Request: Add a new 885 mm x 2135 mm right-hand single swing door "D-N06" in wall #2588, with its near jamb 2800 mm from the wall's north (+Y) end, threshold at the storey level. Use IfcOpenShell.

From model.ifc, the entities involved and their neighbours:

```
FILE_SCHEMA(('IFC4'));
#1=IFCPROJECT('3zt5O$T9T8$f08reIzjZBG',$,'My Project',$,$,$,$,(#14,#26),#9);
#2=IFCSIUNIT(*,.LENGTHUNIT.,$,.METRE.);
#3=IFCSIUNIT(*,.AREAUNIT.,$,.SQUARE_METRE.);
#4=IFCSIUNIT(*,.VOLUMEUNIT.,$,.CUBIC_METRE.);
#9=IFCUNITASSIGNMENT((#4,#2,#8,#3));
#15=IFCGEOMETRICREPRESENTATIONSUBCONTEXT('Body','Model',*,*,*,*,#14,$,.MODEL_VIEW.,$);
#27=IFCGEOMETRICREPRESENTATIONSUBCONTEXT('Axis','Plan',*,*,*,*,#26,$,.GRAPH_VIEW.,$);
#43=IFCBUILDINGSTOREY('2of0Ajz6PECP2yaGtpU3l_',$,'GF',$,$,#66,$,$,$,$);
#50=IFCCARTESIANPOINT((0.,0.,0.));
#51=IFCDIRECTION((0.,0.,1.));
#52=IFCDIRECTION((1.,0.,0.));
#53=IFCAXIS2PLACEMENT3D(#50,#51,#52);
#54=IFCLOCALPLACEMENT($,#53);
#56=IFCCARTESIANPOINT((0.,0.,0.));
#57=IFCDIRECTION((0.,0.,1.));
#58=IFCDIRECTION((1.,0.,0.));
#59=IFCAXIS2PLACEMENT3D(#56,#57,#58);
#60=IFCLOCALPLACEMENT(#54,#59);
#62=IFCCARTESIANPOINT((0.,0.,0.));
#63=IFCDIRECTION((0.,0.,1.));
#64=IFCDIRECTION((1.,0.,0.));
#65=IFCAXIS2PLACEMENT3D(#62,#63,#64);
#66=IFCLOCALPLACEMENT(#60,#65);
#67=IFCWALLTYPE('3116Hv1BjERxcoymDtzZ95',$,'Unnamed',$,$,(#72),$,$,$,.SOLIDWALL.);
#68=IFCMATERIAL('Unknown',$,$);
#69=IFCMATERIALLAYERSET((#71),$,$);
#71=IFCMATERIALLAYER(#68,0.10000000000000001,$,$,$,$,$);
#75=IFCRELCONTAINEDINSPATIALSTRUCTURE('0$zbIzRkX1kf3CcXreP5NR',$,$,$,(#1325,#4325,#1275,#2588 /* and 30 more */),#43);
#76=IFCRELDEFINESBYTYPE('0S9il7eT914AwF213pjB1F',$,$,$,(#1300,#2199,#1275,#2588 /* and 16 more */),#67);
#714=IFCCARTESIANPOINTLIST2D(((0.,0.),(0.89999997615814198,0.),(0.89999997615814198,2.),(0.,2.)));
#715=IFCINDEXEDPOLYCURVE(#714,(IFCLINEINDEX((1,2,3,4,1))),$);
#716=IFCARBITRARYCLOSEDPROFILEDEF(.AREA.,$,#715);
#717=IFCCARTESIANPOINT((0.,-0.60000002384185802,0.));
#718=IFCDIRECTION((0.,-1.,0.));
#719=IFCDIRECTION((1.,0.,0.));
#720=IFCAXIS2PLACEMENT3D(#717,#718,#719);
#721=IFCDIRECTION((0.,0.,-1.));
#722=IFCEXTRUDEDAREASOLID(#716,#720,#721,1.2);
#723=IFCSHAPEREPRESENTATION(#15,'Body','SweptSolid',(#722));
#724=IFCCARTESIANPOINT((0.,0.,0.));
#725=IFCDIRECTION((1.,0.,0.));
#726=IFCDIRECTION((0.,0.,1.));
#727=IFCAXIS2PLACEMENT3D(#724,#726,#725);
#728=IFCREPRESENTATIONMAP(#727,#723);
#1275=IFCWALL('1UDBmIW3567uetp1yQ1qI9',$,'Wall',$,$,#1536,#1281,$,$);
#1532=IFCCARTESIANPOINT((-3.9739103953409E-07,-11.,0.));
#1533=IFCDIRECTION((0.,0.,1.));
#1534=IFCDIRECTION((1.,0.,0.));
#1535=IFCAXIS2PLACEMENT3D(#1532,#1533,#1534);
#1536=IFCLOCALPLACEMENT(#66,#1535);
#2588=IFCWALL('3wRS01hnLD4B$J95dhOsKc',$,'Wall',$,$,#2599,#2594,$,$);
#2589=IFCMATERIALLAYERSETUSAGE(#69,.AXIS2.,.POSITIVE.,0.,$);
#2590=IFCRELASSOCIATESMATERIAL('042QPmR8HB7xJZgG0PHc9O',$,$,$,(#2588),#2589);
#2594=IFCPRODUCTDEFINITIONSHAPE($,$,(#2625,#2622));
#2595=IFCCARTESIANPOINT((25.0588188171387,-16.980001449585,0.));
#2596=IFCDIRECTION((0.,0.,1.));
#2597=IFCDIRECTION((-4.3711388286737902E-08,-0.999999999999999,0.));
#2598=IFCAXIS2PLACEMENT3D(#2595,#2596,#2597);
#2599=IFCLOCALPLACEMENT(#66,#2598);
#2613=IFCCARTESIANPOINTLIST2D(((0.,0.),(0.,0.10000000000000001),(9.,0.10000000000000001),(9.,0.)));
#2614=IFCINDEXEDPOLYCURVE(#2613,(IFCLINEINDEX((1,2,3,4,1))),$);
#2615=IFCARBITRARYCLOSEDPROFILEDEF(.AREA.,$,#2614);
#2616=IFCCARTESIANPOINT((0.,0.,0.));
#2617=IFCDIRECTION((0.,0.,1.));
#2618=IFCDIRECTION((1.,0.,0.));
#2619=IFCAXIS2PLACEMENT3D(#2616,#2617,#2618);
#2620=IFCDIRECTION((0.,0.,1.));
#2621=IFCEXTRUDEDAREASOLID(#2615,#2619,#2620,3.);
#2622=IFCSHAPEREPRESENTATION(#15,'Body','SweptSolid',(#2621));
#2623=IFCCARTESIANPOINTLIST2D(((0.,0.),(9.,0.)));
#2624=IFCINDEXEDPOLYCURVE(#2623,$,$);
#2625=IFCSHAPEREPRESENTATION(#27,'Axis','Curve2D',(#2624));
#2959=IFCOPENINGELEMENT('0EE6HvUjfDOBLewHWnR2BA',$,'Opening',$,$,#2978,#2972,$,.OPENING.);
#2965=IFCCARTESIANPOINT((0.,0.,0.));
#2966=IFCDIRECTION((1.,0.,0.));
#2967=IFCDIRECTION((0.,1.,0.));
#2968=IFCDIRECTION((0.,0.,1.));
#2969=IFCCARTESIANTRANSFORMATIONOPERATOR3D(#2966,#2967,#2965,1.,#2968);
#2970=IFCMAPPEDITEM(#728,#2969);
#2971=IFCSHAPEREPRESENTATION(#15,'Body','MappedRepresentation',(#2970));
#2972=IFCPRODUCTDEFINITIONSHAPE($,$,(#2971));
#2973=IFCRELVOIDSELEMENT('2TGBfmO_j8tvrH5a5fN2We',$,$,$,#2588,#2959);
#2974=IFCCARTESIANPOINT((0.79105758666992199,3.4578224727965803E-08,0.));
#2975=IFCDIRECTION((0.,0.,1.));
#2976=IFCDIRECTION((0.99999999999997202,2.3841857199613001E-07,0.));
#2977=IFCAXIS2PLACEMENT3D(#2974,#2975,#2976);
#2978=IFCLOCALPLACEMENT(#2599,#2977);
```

```python
import numpy as np
import ifcopenshell
import ifcopenshell.api.feature
import ifcopenshell.api.geometry
import ifcopenshell.api.root
import ifcopenshell.api.spatial
import ifcopenshell.geom
import ifcopenshell.util.element
import ifcopenshell.util.placement
import ifcopenshell.util.representation
import ifcopenshell.util.shape
import ifcopenshell.util.unit

model = ifcopenshell.open("model.ifc")
unit_scale = ifcopenshell.util.unit.calculate_unit_scale(model)
settings = ifcopenshell.geom.settings()


def volume(element):
    """Net volume in cubic metres, openings subtracted."""
    shape = ifcopenshell.geom.create_shape(settings, element)
    return ifcopenshell.util.shape.get_volume(shape.geometry)


wall = model.by_id(2588)
storey = ifcopenshell.util.element.get_container(wall, ifc_class="IfcBuildingStorey")
context = ifcopenshell.util.representation.get_context(model, "Model", "Body", "MODEL_VIEW")
before = volume(wall)

width, height, from_end, sill = 0.885, 2.135, 2.8, 0.0  # metres

# The wall runs along its own X axis, and the end named is its -X end.
wall_shape = ifcopenshell.geom.create_shape(settings, wall)
x, y, z = ifcopenshell.util.shape.get_vertices(wall_shape.geometry).T
start = x.min() + from_end
face, thickness = float(y.min()), float(y.max() - y.min())
wall_matrix = ifcopenshell.util.placement.get_local_placement(wall.ObjectPlacement)
level = ifcopenshell.util.placement.get_local_placement(storey.ObjectPlacement)[2, 3]


def in_wall(x, y):
    """Placement at x, y metres in the wall's axes, at sill height."""
    matrix = wall_matrix.copy()
    matrix[:, 3] = wall_matrix @ np.array([x / unit_scale, y / unit_scale, 0.0, 1.0])
    matrix[2, 3] = level + sill / unit_scale
    return matrix


# Opening: a box that overshoots both wall faces by 50 mm.
opening = ifcopenshell.api.root.create_entity(model, ifc_class="IfcOpeningElement", predefined_type="OPENING")
box = ifcopenshell.api.geometry.add_wall_representation(
    model, context=context, length=width, height=height, thickness=thickness + 0.1
)
ifcopenshell.api.geometry.assign_representation(model, product=opening, representation=box)
ifcopenshell.api.geometry.edit_object_placement(model, product=opening, matrix=in_wall(start, face - 0.05), is_si=False)
ifcopenshell.api.feature.add_feature(model, feature=opening, element=wall)

door = ifcopenshell.api.root.create_entity(model, ifc_class="IfcDoor", name="D-N06", predefined_type="DOOR")
door.OverallWidth, door.OverallHeight = width / unit_scale, height / unit_scale
door.OperationType = "SINGLE_SWING_RIGHT"
body = ifcopenshell.api.geometry.add_door_representation(
    model,
    context=context,
    overall_width=door.OverallWidth,
    overall_height=door.OverallHeight,
    operation_type="SINGLE_SWING_RIGHT",
    lining_properties={"LiningDepth": thickness / unit_scale, "ThresholdDepth": thickness / unit_scale},
)
ifcopenshell.api.geometry.assign_representation(model, product=door, representation=body)
ifcopenshell.api.spatial.assign_container(model, products=[door], relating_structure=storey)
ifcopenshell.api.feature.add_filling(model, opening=opening, element=door)

# The lining spans the wall, so the door starts at the wall face.
ifcopenshell.api.geometry.edit_object_placement(model, product=door, matrix=in_wall(start, face), is_si=False)

after = volume(wall)

print(f"wall volume {before:.3f} -> {after:.3f} m3")

model.write("model_updated.ifc")
```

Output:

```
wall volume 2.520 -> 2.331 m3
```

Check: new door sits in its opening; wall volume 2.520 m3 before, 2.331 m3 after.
